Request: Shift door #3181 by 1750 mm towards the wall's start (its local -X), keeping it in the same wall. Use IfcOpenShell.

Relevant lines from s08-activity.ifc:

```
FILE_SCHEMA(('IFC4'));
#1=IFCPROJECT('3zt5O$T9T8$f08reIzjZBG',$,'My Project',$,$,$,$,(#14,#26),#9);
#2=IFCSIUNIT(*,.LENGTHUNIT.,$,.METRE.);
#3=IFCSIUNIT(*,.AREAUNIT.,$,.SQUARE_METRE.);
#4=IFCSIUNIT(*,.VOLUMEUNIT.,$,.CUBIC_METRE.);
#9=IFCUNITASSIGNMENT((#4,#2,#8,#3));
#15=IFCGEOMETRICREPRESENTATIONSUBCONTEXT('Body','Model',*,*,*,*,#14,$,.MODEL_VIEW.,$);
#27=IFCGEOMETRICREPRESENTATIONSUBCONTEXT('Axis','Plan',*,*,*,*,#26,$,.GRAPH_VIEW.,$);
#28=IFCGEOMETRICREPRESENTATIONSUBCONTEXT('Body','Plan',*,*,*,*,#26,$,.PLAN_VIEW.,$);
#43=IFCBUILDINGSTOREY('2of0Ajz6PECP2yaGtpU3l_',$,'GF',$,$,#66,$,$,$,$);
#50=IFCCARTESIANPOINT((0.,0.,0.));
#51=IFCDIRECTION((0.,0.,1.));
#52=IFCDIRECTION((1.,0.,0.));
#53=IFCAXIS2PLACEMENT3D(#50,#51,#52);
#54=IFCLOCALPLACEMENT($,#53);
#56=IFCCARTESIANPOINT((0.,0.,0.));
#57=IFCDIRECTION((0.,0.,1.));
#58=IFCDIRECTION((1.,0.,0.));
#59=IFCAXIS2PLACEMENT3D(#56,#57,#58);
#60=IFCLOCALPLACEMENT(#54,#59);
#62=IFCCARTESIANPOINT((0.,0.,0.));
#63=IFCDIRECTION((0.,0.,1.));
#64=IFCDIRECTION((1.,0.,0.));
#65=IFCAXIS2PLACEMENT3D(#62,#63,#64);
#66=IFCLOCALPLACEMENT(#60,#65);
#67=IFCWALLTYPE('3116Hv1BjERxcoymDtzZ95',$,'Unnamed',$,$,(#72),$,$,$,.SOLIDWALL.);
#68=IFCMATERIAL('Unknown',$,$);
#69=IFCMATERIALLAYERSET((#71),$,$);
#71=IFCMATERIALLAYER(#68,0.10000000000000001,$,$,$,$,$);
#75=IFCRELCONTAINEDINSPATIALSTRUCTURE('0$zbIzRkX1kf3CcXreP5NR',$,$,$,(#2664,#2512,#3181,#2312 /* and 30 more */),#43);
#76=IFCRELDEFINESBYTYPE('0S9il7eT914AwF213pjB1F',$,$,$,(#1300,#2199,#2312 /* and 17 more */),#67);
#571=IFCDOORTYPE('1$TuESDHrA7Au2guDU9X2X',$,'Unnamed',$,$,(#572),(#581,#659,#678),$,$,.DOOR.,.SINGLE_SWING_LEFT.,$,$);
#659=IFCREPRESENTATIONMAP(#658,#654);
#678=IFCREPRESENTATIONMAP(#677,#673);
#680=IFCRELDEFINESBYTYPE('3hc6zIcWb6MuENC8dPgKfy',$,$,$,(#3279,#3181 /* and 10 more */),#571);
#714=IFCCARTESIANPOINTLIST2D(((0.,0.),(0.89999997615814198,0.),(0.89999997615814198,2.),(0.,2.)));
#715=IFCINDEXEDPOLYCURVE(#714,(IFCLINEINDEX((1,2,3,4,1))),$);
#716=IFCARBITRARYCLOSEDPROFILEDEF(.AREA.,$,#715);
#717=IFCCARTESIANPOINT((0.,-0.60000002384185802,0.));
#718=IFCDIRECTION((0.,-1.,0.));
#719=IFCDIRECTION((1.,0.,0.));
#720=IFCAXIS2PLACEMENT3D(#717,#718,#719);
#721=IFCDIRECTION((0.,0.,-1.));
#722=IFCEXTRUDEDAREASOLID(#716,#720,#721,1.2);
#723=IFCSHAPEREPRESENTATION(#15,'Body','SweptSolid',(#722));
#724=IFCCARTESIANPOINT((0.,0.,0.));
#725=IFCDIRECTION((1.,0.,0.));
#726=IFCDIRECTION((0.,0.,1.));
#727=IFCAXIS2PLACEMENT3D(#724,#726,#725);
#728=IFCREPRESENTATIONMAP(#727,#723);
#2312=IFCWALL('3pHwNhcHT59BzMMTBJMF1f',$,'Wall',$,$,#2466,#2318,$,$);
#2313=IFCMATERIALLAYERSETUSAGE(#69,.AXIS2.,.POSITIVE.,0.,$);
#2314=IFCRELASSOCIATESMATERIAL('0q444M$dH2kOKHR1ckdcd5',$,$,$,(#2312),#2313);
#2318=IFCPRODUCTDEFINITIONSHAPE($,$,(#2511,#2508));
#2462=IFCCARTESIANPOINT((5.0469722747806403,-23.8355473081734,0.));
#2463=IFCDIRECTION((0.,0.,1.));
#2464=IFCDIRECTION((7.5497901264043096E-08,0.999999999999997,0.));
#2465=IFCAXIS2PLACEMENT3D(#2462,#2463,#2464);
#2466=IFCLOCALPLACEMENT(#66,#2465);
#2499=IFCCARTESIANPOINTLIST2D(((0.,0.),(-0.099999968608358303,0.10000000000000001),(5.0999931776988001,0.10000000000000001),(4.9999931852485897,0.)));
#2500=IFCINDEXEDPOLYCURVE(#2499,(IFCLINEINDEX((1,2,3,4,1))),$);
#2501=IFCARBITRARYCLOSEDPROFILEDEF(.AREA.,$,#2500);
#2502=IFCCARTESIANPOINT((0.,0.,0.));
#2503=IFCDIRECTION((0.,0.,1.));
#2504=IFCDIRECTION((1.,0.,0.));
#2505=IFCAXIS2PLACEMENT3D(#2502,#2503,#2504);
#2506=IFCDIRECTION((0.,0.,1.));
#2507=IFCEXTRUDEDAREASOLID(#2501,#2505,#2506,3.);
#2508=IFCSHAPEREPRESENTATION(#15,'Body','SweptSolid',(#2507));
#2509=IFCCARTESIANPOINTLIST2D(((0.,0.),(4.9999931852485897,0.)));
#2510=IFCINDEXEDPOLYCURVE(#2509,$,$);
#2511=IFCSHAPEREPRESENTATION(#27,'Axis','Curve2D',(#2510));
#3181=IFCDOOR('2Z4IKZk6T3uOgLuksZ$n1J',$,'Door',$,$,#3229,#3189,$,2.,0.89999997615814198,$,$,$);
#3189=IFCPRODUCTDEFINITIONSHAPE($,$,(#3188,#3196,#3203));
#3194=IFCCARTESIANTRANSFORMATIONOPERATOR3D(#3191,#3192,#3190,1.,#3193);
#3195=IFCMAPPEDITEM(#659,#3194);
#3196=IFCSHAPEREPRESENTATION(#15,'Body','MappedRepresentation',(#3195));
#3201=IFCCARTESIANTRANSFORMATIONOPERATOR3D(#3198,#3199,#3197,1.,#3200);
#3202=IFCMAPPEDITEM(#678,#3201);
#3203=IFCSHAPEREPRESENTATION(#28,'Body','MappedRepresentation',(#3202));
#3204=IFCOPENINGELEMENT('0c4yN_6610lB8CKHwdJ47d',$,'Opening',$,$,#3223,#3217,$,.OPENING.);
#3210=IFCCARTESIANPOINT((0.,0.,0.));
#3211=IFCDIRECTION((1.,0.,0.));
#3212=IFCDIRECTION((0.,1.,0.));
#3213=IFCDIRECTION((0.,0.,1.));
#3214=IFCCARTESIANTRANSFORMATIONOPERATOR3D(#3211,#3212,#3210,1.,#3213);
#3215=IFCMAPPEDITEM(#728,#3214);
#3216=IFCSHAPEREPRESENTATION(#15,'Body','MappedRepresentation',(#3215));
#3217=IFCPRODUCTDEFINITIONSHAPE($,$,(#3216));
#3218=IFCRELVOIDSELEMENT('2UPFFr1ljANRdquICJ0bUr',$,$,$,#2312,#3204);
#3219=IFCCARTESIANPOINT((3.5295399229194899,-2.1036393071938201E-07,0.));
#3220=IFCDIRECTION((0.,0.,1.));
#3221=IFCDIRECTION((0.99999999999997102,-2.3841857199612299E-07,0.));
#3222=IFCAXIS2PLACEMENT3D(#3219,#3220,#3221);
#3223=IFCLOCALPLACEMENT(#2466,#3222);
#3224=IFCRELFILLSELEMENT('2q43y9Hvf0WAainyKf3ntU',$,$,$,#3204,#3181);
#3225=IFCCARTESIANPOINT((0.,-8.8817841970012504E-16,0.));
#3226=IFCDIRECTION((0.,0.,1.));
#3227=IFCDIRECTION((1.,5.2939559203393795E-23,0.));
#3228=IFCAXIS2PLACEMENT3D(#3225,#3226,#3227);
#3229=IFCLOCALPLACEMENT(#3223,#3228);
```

```python
import ifcopenshell
import ifcopenshell.api.geometry
import ifcopenshell.util.placement
import ifcopenshell.util.unit

model = ifcopenshell.open("s08-activity.ifc")
unit_scale = ifcopenshell.util.unit.calculate_unit_scale(model)

door = model.by_id(3181)
opening = door.FillsVoids[0].RelatingOpeningElement
wall = opening.VoidsElements[0].RelatingBuildingElement

wall_matrix = ifcopenshell.util.placement.get_local_placement(wall.ObjectPlacement)
shift = wall_matrix[:3, 0] * -1.75 / unit_scale
before = ifcopenshell.util.placement.get_local_placement(door.ObjectPlacement)[:3, 3].copy()

# The door is placed relative to its opening, so it follows when the opening moves.
matrix = ifcopenshell.util.placement.get_local_placement(opening.ObjectPlacement)
matrix[:3, 3] += shift
ifcopenshell.api.geometry.edit_object_placement(
    model, product=opening, matrix=matrix, is_si=False, should_transform_children=True
)

after = ifcopenshell.util.placement.get_local_placement(door.ObjectPlacement)[:3, 3]
print("door moved by", (after - before).round(3) + 0.0)

model.write("s08-activity_rev.ifc")
```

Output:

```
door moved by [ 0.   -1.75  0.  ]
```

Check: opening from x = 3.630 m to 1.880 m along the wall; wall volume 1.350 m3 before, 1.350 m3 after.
